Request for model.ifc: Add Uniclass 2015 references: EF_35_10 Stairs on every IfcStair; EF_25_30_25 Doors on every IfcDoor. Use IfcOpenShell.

First a look at what the model holds.

```python
import ifcopenshell

model = ifcopenshell.open("model.ifc")
print(model.schema)
print("classifications:", [c.Name for c in model.by_type("IfcClassification")])
for ifc_class in ("IfcDoor", "IfcRoof", "IfcStair", "IfcWall", "IfcWindow"):
    print(ifc_class, len(model.by_type(ifc_class)))
```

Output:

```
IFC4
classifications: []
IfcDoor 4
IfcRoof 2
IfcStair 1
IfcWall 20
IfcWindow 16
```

```python
import ifcopenshell
import ifcopenshell.api.classification

model = ifcopenshell.open("model.ifc")

system = ifcopenshell.api.classification.add_classification(model, classification="Uniclass 2015")

codes = {
    "IfcStair": ("EF_35_10", "Stairs"),
    "IfcDoor": ("EF_25_30_25", "Doors"),
}
for ifc_class, (code, name) in codes.items():
    products = model.by_type(ifc_class)
    ifcopenshell.api.classification.add_reference(
        model, products=products, classification=system, identification=code, name=name
    )
    print(code, len(products))

model.write("model_edited.ifc")
```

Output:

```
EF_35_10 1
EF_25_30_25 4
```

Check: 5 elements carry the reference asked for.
